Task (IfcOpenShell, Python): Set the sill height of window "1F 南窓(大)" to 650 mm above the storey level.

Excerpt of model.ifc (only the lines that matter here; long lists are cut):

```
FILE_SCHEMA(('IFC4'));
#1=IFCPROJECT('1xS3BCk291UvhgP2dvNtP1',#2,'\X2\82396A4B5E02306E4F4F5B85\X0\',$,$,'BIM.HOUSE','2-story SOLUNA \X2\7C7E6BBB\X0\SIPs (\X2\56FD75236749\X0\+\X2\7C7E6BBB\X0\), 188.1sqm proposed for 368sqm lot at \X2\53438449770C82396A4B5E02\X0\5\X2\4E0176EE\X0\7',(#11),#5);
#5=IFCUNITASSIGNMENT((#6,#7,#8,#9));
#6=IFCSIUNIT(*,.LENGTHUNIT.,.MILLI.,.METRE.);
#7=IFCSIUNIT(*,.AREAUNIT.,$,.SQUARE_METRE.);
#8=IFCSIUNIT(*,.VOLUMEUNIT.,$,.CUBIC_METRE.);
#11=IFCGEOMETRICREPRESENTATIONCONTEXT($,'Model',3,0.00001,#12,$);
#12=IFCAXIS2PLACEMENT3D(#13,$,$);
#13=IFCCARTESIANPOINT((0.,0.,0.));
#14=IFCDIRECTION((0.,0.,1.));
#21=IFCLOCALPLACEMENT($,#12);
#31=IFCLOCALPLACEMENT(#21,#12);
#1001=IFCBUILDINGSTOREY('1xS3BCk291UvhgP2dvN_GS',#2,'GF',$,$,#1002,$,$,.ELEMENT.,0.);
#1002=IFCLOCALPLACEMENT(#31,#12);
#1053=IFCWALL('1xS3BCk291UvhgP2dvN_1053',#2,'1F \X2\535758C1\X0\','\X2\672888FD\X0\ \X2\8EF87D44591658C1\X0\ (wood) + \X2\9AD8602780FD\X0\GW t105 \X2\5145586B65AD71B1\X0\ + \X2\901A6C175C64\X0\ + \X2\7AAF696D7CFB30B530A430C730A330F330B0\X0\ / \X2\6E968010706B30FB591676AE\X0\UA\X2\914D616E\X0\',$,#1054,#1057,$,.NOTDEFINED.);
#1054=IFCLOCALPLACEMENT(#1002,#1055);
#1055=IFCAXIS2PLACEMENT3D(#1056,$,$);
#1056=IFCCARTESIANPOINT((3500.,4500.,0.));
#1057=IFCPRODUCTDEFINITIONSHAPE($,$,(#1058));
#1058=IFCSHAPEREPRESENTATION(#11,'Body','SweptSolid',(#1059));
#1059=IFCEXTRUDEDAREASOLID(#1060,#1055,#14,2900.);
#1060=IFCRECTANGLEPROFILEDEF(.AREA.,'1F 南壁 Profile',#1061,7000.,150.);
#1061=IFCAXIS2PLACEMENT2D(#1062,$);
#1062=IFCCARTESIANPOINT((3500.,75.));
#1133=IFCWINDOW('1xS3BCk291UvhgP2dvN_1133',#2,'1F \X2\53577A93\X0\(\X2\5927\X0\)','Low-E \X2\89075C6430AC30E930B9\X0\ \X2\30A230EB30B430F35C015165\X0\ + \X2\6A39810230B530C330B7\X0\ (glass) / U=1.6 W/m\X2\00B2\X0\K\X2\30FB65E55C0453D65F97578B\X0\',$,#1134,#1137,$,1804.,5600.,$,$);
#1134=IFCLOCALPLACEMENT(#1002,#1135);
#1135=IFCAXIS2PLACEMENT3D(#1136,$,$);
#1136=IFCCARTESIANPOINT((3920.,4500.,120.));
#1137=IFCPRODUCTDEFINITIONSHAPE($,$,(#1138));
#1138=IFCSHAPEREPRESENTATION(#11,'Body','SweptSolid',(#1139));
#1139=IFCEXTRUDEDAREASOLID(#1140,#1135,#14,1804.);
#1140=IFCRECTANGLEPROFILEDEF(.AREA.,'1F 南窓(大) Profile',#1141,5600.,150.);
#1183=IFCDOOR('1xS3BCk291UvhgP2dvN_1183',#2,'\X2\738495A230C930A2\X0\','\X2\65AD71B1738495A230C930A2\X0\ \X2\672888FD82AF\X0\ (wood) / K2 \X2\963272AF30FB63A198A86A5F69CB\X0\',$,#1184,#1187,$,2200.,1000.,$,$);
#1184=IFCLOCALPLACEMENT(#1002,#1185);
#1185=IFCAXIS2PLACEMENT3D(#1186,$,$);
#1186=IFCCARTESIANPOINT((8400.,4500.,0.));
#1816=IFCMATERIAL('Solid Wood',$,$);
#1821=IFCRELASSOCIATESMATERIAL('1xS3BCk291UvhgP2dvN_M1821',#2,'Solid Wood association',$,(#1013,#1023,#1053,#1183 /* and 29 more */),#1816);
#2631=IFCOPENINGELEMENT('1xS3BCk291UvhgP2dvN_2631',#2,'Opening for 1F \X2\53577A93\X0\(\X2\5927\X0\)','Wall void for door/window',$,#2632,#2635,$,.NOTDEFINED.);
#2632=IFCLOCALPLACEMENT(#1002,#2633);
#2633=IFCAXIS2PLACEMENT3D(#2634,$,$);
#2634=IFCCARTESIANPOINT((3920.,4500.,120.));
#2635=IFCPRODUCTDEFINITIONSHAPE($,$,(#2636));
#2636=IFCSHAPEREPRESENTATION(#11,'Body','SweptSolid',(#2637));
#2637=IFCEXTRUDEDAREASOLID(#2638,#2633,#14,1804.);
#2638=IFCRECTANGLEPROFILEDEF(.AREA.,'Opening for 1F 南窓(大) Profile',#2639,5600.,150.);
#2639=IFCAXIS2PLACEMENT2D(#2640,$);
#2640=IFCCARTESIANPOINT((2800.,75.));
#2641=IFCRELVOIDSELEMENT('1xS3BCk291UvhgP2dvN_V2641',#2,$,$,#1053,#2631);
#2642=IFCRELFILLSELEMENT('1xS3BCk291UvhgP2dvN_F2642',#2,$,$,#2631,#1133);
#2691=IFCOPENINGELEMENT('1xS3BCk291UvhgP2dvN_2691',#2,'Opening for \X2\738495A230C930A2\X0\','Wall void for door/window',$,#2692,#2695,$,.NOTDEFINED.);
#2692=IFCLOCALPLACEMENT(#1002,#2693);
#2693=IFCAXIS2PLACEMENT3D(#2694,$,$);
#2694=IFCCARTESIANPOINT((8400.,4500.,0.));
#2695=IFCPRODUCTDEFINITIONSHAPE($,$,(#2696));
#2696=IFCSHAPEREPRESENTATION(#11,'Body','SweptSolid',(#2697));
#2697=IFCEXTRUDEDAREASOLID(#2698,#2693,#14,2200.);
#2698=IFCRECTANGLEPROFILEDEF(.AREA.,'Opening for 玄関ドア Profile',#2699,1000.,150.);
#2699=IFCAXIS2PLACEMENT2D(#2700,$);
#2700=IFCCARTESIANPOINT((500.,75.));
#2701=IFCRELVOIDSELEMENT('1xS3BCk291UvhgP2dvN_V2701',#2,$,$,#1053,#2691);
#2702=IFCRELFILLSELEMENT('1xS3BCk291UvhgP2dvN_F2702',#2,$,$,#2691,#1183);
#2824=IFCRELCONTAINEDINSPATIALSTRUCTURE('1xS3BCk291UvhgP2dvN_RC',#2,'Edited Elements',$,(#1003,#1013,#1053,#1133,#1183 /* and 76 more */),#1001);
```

```python
import numpy as np
import ifcopenshell
import ifcopenshell.api.geometry
import ifcopenshell.geom
import ifcopenshell.util.element
import ifcopenshell.util.placement
import ifcopenshell.util.shape
import ifcopenshell.util.unit

model = ifcopenshell.open("model.ifc")
unit_scale = ifcopenshell.util.unit.calculate_unit_scale(model)

window = model.by_guid("1xS3BCk291UvhgP2dvN_1133")
opening = window.FillsVoids[0].RelatingOpeningElement
storey = ifcopenshell.util.element.get_container(window, ifc_class="IfcBuildingStorey")
level = ifcopenshell.util.placement.get_local_placement(storey.ObjectPlacement)[2, 3]

# The opening's origin need not be at the sill, so measure its lowest point.
shape = ifcopenshell.geom.create_shape(ifcopenshell.geom.settings(), opening)
bottom = ifcopenshell.util.shape.get_shape_bottom_elevation(shape, shape.geometry) / unit_scale
dz = level + 0.65 / unit_scale - bottom

shift = np.array([0.0, 0.0, dz])
# The window is not placed relative to its opening, so move both.
for product in (opening, window):
    matrix = ifcopenshell.util.placement.get_local_placement(product.ObjectPlacement)
    matrix[:3, 3] += shift
    ifcopenshell.api.geometry.edit_object_placement(model, product=product, matrix=matrix, is_si=False)

print(f"moved by {dz * unit_scale:+.3f} m")

model.write("model-out.ifc")
```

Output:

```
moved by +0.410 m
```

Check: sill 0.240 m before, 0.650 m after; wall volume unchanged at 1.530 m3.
